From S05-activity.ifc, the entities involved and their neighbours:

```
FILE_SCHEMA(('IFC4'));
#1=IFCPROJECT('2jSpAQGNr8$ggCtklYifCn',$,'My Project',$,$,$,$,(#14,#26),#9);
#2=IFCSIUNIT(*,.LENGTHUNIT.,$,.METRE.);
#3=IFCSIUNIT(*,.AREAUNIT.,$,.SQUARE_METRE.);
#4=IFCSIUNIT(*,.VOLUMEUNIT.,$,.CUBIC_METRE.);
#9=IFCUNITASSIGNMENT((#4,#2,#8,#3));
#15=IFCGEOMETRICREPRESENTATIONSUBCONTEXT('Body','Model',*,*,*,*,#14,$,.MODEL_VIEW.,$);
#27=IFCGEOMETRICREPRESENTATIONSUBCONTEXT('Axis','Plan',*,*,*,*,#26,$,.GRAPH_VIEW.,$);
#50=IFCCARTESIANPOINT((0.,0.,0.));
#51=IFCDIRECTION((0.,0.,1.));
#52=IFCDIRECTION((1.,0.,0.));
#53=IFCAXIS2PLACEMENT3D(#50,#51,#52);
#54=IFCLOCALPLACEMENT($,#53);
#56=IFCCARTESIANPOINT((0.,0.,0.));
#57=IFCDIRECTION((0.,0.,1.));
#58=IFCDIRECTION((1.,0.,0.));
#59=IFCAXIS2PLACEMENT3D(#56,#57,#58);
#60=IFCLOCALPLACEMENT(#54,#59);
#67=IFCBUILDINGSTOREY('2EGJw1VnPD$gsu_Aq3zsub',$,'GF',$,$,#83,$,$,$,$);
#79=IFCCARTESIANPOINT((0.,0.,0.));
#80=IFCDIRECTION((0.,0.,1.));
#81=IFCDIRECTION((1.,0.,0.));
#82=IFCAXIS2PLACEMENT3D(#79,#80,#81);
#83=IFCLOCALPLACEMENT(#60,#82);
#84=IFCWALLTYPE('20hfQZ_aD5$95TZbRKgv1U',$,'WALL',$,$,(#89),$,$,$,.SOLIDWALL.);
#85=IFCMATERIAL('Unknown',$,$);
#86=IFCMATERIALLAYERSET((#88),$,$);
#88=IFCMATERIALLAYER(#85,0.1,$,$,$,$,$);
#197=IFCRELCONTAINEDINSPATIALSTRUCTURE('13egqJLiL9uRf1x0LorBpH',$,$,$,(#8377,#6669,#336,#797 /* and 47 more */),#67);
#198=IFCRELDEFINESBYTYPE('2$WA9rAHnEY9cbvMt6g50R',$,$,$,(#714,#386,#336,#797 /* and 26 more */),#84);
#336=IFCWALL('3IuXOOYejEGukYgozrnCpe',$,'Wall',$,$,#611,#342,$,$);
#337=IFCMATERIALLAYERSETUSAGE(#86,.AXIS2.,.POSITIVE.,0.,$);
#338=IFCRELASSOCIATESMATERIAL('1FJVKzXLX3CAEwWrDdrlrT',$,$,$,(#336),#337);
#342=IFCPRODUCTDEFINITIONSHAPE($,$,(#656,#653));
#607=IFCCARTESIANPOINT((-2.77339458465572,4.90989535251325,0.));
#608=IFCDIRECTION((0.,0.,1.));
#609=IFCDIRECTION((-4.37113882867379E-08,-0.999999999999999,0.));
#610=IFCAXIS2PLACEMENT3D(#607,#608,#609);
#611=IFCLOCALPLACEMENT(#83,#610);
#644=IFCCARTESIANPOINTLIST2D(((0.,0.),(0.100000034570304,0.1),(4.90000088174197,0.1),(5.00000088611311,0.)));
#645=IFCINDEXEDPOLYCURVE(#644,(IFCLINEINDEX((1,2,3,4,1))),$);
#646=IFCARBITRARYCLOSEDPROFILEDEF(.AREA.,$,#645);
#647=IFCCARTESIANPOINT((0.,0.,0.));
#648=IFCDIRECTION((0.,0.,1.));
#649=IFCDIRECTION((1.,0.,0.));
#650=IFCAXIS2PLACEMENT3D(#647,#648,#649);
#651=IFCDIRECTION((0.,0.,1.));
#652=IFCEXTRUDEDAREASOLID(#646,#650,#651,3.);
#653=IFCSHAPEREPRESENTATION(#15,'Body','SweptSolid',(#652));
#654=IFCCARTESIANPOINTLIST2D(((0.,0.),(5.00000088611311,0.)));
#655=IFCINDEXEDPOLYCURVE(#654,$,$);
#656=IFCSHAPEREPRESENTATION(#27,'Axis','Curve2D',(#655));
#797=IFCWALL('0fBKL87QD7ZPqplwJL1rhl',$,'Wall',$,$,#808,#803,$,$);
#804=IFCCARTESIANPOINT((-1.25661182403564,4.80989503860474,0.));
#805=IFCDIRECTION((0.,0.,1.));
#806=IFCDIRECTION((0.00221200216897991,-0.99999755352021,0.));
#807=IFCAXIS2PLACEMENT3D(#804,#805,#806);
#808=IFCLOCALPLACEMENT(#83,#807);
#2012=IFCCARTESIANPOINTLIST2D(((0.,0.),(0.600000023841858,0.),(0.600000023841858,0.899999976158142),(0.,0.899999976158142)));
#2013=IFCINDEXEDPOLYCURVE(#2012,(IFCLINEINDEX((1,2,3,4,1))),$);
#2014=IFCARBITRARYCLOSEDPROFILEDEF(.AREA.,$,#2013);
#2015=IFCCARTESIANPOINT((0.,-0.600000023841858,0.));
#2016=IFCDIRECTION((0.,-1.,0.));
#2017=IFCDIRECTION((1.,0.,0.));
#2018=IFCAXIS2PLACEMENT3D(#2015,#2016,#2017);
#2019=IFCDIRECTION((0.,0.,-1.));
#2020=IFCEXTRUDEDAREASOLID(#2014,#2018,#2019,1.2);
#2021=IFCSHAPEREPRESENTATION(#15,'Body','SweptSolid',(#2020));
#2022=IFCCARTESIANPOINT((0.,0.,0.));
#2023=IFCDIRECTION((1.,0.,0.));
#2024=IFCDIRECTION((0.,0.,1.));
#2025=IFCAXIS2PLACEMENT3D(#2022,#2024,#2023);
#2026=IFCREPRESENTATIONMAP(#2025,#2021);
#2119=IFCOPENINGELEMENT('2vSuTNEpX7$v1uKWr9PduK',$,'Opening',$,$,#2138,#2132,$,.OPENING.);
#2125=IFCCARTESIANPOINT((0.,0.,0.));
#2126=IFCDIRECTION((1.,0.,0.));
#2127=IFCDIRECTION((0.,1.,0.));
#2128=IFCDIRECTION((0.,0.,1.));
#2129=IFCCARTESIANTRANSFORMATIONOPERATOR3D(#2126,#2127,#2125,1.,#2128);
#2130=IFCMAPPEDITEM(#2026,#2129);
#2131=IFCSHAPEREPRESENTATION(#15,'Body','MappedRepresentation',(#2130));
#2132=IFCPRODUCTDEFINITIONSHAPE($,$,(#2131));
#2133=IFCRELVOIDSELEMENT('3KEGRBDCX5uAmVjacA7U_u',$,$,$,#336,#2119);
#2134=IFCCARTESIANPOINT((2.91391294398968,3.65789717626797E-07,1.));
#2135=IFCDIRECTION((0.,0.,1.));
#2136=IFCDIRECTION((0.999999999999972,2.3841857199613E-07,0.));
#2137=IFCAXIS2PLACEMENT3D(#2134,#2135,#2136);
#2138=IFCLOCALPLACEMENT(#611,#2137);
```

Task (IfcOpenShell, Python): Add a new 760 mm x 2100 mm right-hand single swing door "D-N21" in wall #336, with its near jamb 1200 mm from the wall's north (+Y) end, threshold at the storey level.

```python
import numpy as np
import ifcopenshell
import ifcopenshell.api.feature
import ifcopenshell.api.geometry
import ifcopenshell.api.root
import ifcopenshell.api.spatial
import ifcopenshell.geom
import ifcopenshell.util.element
import ifcopenshell.util.placement
import ifcopenshell.util.representation
import ifcopenshell.util.shape
import ifcopenshell.util.unit

model = ifcopenshell.open("S05-activity.ifc")
unit_scale = ifcopenshell.util.unit.calculate_unit_scale(model)
settings = ifcopenshell.geom.settings()


def volume(element):
    """Net volume in cubic metres, openings subtracted."""
    shape = ifcopenshell.geom.create_shape(settings, element)
    return ifcopenshell.util.shape.get_volume(shape.geometry)


wall = model.by_id(336)
storey = ifcopenshell.util.element.get_container(wall, ifc_class="IfcBuildingStorey")
context = ifcopenshell.util.representation.get_context(model, "Model", "Body", "MODEL_VIEW")
before = volume(wall)

width, height, from_end, sill = 0.76, 2.1, 1.2, 0.0  # metres

# The wall runs along its own X axis, and the end named is its -X end.
wall_shape = ifcopenshell.geom.create_shape(settings, wall)
x, y, z = ifcopenshell.util.shape.get_vertices(wall_shape.geometry).T
start = x.min() + from_end
face, thickness = float(y.min()), float(y.max() - y.min())
wall_matrix = ifcopenshell.util.placement.get_local_placement(wall.ObjectPlacement)
level = ifcopenshell.util.placement.get_local_placement(storey.ObjectPlacement)[2, 3]


def in_wall(x, y):
    """Placement at x, y metres in the wall's axes, at sill height."""
    matrix = wall_matrix.copy()
    matrix[:, 3] = wall_matrix @ np.array([x / unit_scale, y / unit_scale, 0.0, 1.0])
    matrix[2, 3] = level + sill / unit_scale
    return matrix


# Opening: a box that overshoots both wall faces by 50 mm.
opening = ifcopenshell.api.root.create_entity(model, ifc_class="IfcOpeningElement", predefined_type="OPENING")
box = ifcopenshell.api.geometry.add_wall_representation(
    model, context=context, length=width, height=height, thickness=thickness + 0.1
)
ifcopenshell.api.geometry.assign_representation(model, product=opening, representation=box)
ifcopenshell.api.geometry.edit_object_placement(model, product=opening, matrix=in_wall(start, face - 0.05), is_si=False)
ifcopenshell.api.feature.add_feature(model, feature=opening, element=wall)

door = ifcopenshell.api.root.create_entity(model, ifc_class="IfcDoor", name="D-N21", predefined_type="DOOR")
door.OverallWidth, door.OverallHeight = width / unit_scale, height / unit_scale
door.OperationType = "SINGLE_SWING_RIGHT"
body = ifcopenshell.api.geometry.add_door_representation(
    model,
    context=context,
    overall_width=door.OverallWidth,
    overall_height=door.OverallHeight,
    operation_type="SINGLE_SWING_RIGHT",
    lining_properties={"LiningDepth": thickness / unit_scale, "ThresholdDepth": thickness / unit_scale},
)
ifcopenshell.api.geometry.assign_representation(model, product=door, representation=body)
ifcopenshell.api.spatial.assign_container(model, products=[door], relating_structure=storey)
ifcopenshell.api.feature.add_filling(model, opening=opening, element=door)

# The lining spans the wall, so the door starts at the wall face.
ifcopenshell.api.geometry.edit_object_placement(model, product=door, matrix=in_wall(start, face), is_si=False)

after = volume(wall)

print(f"wall volume {before:.3f} -> {after:.3f} m3")

model.write("S05-activity_edited.ifc")
```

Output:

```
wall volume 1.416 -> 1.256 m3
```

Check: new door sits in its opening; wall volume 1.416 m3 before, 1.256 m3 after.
